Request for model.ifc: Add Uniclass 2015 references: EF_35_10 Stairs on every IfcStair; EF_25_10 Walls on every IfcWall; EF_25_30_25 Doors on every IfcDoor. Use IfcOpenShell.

First a look at what the model holds.

```python
import ifcopenshell

model = ifcopenshell.open("model.ifc")
print(model.schema)
print("classifications:", [c.Name for c in model.by_type("IfcClassification")])
for ifc_class in ("IfcDoor", "IfcRoof", "IfcStair", "IfcWall", "IfcWindow"):
    print(ifc_class, len(model.by_type(ifc_class)))
```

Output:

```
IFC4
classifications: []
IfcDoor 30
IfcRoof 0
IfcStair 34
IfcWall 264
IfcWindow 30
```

```python
import ifcopenshell
import ifcopenshell.api.classification

model = ifcopenshell.open("model.ifc")

system = ifcopenshell.api.classification.add_classification(model, classification="Uniclass 2015")

codes = {
    "IfcStair": ("EF_35_10", "Stairs"),
    "IfcWall": ("EF_25_10", "Walls"),
    "IfcDoor": ("EF_25_30_25", "Doors"),
}
for ifc_class, (code, name) in codes.items():
    products = model.by_type(ifc_class)
    ifcopenshell.api.classification.add_reference(
        model, products=products, classification=system, identification=code, name=name
    )
    print(code, len(products))

model.write("model_edited.ifc")
```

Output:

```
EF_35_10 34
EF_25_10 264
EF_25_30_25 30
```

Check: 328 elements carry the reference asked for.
